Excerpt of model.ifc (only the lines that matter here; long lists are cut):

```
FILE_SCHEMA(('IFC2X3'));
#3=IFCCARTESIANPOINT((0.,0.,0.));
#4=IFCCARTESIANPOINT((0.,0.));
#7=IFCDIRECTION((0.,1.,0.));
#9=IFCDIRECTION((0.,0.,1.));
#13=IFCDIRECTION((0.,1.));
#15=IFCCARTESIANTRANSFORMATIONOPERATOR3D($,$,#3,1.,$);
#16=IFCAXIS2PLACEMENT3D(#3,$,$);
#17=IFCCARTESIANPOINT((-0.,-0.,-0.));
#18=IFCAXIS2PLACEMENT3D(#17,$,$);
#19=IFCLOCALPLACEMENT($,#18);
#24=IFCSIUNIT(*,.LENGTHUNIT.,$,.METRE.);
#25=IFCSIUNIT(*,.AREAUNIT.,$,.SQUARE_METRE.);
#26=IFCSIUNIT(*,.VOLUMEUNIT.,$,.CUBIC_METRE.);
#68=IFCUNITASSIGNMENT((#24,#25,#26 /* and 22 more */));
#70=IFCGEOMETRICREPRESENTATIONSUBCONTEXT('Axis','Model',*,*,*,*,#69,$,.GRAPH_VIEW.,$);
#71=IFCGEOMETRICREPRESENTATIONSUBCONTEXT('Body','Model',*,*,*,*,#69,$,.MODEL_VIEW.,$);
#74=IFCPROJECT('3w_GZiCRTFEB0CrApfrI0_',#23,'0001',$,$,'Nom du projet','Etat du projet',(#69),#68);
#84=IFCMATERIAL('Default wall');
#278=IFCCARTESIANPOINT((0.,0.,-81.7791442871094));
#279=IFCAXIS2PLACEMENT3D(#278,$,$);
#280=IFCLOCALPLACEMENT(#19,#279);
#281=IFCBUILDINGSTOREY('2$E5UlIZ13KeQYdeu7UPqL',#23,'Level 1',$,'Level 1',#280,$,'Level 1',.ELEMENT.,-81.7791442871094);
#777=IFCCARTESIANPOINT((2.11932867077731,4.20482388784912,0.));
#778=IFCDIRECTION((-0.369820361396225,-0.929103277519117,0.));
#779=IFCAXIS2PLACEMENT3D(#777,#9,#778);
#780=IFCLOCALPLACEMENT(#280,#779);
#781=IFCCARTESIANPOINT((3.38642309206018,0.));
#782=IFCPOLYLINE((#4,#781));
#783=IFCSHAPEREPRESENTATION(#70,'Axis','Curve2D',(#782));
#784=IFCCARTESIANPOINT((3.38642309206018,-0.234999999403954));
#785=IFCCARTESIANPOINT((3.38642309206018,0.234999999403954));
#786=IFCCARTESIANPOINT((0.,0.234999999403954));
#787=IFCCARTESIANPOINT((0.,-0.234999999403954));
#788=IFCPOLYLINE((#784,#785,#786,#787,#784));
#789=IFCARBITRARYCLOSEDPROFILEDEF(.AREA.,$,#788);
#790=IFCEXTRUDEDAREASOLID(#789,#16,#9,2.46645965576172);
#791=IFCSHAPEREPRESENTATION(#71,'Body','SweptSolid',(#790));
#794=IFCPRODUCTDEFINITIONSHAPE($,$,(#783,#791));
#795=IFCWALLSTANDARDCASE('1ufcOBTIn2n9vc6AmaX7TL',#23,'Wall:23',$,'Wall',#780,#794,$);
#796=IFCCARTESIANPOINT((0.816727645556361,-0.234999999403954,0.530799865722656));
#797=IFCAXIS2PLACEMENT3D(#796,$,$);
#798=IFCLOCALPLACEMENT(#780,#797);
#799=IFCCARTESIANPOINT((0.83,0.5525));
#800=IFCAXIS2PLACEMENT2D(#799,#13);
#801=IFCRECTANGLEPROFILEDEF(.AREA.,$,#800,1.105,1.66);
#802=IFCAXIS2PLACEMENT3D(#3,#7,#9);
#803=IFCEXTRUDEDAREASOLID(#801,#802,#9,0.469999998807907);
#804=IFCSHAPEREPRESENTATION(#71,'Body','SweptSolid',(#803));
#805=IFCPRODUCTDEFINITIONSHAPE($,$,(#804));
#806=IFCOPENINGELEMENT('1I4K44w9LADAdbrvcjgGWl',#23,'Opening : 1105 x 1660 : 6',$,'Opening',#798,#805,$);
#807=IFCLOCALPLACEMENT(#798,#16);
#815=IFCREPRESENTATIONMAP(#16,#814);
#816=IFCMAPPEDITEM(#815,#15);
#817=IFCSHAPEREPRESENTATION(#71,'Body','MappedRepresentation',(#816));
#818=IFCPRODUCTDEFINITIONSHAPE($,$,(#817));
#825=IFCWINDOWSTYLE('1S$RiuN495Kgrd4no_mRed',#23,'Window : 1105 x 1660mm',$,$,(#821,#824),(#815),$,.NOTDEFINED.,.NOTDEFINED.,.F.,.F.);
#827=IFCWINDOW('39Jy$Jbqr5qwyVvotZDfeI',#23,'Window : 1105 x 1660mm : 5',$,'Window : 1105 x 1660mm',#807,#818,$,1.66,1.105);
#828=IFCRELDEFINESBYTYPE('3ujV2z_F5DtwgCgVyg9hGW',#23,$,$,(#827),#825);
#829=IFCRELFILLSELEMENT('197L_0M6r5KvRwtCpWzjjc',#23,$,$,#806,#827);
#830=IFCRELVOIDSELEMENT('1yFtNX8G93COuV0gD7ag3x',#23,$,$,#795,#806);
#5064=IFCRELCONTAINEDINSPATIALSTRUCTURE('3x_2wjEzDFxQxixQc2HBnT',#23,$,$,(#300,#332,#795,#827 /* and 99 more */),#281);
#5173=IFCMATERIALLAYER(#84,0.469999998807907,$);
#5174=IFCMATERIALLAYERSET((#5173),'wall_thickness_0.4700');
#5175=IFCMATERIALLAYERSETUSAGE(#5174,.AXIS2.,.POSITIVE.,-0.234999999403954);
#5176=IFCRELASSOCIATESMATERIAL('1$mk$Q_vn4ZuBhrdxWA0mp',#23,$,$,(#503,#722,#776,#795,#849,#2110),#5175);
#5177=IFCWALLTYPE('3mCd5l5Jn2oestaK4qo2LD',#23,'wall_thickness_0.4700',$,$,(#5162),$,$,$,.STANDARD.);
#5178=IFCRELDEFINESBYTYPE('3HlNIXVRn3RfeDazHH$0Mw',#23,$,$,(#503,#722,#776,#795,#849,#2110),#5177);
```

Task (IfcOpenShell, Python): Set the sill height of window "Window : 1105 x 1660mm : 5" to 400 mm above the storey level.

```python
import numpy as np
import ifcopenshell
import ifcopenshell.api.geometry
import ifcopenshell.geom
import ifcopenshell.util.element
import ifcopenshell.util.placement
import ifcopenshell.util.shape
import ifcopenshell.util.unit

model = ifcopenshell.open("model.ifc")
unit_scale = ifcopenshell.util.unit.calculate_unit_scale(model)

window = model.by_id(827)
opening = window.FillsVoids[0].RelatingOpeningElement
storey = ifcopenshell.util.element.get_container(window, ifc_class="IfcBuildingStorey")
level = ifcopenshell.util.placement.get_local_placement(storey.ObjectPlacement)[2, 3]

# The opening's origin need not be at the sill, so measure its lowest point.
shape = ifcopenshell.geom.create_shape(ifcopenshell.geom.settings(), opening)
bottom = ifcopenshell.util.shape.get_shape_bottom_elevation(shape, shape.geometry) / unit_scale
dz = level + 0.4 / unit_scale - bottom

shift = np.array([0.0, 0.0, dz])
# The window is placed relative to its opening, so it follows when the opening moves.
matrix = ifcopenshell.util.placement.get_local_placement(opening.ObjectPlacement)
matrix[:3, 3] += shift
ifcopenshell.api.geometry.edit_object_placement(
    model, product=opening, matrix=matrix, is_si=False, should_transform_children=True
)

print(f"moved by {dz * unit_scale:+.3f} m")

model.write("model_v2.ifc")
```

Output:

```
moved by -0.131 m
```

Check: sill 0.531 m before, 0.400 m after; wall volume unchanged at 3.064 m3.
